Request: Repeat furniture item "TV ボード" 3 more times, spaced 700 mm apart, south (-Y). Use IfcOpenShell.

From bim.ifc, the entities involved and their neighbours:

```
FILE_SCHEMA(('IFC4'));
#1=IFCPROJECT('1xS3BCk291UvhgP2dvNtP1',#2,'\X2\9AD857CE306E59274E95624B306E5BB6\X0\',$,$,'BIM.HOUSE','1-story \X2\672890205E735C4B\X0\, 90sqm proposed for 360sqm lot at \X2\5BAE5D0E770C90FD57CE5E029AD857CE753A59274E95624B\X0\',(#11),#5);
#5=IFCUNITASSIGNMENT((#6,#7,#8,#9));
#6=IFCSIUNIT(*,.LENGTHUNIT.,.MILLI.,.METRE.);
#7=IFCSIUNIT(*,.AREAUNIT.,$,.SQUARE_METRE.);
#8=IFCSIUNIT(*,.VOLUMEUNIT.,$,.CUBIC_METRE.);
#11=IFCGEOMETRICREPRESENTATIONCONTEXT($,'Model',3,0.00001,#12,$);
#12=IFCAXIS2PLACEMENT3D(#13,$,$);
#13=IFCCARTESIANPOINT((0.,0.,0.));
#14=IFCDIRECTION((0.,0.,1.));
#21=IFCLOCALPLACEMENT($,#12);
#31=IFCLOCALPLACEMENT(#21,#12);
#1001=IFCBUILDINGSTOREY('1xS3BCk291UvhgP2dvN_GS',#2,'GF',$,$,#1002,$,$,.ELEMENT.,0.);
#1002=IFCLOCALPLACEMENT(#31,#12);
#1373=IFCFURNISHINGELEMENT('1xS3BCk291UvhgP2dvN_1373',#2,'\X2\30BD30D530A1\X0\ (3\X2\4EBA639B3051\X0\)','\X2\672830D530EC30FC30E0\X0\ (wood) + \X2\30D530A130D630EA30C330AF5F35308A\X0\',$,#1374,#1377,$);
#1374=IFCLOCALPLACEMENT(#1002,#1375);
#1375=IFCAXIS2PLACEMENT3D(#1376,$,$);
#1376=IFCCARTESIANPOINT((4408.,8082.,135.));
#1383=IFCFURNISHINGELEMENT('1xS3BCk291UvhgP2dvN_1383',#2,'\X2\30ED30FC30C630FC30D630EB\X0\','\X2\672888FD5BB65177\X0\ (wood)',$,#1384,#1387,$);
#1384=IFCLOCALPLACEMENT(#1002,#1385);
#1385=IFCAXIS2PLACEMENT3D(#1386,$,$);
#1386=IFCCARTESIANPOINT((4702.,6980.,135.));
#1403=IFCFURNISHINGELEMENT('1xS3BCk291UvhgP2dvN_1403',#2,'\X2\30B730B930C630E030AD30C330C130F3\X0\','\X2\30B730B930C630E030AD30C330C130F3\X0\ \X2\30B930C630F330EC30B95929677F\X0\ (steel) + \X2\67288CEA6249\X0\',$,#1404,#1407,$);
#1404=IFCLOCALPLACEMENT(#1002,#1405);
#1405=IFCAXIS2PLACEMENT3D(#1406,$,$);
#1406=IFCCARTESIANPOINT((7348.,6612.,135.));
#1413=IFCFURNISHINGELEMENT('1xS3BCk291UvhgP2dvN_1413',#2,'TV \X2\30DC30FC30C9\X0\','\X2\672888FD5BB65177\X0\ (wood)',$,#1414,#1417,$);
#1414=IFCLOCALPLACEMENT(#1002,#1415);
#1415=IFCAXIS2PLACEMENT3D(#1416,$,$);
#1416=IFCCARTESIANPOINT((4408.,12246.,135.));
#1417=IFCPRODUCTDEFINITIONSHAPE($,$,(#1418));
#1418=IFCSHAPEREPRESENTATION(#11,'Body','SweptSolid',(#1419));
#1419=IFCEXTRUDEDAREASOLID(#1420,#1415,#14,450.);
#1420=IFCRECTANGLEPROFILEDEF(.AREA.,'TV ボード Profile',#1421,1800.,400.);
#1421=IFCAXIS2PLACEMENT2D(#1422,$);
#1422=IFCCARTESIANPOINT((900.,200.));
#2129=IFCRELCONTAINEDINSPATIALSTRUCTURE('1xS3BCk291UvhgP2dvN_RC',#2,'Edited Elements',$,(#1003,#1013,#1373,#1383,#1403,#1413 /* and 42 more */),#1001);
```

```python
import numpy as np
import ifcopenshell
import ifcopenshell.api.geometry
import ifcopenshell.api.root
import ifcopenshell.util.element
import ifcopenshell.util.placement

model = ifcopenshell.open("bim.ifc")


def reuse_history(source, copy):
    """copy_class also copies each property set's owner history, people and application; keep the originals."""
    for rel in copy.IsDefinedBy:
        if rel.is_a("IfcRelDefinesByProperties") and (history := rel.RelatingPropertyDefinition.OwnerHistory):
            rel.RelatingPropertyDefinition.OwnerHistory = source.OwnerHistory
            ifcopenshell.util.element.remove_deep2(model, history)


source = model.by_guid("1xS3BCk291UvhgP2dvN_1413")
base = ifcopenshell.util.placement.get_local_placement(source.ObjectPlacement)
step = np.array([0.0, -1.0, 0.0]) * 700.0

for i in range(1, 4):
    copy = ifcopenshell.api.root.copy_class(model, product=source)
    copy.Representation = ifcopenshell.util.element.copy_deep(
        model, source.Representation, exclude=["IfcGeometricRepresentationContext", "IfcRepresentationMap"]
    )
    reuse_history(source, copy)
    matrix = base.copy()
    matrix[:3, 3] += i * step
    print("added at", matrix[:3, 3].round(3) + 0.0)
    ifcopenshell.api.geometry.edit_object_placement(model, product=copy, matrix=matrix, is_si=False)

model.write("bim-out.ifc")
```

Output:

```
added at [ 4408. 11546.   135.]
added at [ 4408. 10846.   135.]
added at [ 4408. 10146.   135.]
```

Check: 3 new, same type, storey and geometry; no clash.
